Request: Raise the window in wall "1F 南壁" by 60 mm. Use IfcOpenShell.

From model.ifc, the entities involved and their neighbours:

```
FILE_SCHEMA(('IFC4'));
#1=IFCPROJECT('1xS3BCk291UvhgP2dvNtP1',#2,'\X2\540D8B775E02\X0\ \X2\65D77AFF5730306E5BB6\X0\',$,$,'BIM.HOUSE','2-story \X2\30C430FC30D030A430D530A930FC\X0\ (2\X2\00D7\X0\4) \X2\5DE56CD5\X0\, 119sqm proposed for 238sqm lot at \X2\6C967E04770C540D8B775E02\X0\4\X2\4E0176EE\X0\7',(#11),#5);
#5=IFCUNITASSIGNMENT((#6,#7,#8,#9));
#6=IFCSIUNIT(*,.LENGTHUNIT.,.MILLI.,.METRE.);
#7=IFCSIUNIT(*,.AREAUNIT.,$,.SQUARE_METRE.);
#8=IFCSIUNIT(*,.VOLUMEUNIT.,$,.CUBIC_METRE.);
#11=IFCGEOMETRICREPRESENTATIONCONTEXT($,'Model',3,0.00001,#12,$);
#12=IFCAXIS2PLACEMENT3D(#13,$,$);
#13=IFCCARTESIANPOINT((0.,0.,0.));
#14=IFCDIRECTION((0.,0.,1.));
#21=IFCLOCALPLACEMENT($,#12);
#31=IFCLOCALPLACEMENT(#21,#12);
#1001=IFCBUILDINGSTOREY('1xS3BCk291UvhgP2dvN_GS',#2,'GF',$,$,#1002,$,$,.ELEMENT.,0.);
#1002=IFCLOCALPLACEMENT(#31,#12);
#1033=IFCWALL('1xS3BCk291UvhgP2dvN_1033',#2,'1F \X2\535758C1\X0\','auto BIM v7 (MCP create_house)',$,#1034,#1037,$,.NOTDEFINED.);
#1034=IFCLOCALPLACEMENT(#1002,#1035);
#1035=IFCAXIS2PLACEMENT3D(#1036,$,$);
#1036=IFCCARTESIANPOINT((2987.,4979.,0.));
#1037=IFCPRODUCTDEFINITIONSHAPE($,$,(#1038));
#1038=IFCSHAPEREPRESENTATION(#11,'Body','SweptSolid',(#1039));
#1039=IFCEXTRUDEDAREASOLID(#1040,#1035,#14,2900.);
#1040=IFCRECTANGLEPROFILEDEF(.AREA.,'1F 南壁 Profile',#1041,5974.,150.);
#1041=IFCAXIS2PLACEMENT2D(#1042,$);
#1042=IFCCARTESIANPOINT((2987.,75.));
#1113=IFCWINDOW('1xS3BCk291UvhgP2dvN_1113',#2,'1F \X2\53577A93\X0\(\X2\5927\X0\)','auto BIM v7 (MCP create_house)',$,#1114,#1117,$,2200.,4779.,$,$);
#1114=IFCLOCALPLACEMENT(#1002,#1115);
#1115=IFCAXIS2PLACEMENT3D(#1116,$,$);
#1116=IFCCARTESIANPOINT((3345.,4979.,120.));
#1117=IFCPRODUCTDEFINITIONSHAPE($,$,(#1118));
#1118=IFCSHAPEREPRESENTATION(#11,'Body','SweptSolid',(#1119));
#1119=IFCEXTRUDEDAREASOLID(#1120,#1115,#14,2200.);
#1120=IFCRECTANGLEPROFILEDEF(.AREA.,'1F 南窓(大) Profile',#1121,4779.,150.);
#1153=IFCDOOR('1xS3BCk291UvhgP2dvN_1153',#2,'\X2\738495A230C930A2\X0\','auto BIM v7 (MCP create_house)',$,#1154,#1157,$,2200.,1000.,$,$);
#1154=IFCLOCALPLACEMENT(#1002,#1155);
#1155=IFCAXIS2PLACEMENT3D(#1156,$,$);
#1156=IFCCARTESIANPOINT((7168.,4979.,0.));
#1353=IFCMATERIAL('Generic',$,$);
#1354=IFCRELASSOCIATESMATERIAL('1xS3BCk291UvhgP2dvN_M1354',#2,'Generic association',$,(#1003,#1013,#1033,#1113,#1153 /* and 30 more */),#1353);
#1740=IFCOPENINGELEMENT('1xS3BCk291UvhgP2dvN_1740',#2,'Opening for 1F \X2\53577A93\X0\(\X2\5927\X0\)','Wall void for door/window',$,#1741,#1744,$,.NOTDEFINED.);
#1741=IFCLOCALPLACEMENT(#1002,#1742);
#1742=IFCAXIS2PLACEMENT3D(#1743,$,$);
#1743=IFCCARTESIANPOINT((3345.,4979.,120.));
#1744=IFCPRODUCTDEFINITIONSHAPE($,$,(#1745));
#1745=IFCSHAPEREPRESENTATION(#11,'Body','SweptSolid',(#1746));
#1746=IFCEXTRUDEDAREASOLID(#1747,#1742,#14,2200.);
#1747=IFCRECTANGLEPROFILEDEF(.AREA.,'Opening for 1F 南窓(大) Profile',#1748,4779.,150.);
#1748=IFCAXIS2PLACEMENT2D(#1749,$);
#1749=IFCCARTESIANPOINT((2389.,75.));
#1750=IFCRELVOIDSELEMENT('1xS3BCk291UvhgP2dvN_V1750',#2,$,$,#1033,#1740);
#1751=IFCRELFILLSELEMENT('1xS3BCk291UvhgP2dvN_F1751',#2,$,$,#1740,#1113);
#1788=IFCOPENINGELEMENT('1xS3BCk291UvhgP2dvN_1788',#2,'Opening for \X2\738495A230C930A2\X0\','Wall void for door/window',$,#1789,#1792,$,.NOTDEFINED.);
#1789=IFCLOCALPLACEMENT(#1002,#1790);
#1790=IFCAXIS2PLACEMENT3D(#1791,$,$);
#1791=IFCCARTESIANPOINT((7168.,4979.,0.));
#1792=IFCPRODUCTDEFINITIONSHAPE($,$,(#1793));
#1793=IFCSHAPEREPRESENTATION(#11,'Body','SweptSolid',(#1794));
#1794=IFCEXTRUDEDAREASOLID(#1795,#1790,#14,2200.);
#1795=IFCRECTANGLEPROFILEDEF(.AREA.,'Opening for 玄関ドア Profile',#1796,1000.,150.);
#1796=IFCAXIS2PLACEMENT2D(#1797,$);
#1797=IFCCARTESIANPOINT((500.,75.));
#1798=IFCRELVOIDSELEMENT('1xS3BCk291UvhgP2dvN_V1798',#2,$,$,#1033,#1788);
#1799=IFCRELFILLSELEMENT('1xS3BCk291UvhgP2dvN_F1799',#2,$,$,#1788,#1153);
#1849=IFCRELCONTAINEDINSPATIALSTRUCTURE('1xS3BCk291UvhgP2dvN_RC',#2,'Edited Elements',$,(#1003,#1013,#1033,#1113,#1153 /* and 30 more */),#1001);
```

```python
import numpy as np
import ifcopenshell
import ifcopenshell.api.geometry
import ifcopenshell.util.placement
import ifcopenshell.util.unit

model = ifcopenshell.open("model.ifc")
unit_scale = ifcopenshell.util.unit.calculate_unit_scale(model)

window = model.by_guid("1xS3BCk291UvhgP2dvN_1113")
opening = window.FillsVoids[0].RelatingOpeningElement
dz = 0.06 / unit_scale

shift = np.array([0.0, 0.0, dz])
# The window is not placed relative to its opening, so move both.
for product in (opening, window):
    matrix = ifcopenshell.util.placement.get_local_placement(product.ObjectPlacement)
    matrix[:3, 3] += shift
    ifcopenshell.api.geometry.edit_object_placement(model, product=product, matrix=matrix, is_si=False)

print(f"moved by {dz * unit_scale:+.3f} m")

model.write("model_updated.ifc")
```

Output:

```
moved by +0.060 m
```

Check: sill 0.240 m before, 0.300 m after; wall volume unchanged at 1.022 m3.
